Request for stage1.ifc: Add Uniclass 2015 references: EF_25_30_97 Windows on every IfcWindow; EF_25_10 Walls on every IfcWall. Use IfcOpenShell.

First a look at what the model holds.

```python
import ifcopenshell

model = ifcopenshell.open("stage1.ifc")
print(model.schema)
print("classifications:", [c.Name for c in model.by_type("IfcClassification")])
for ifc_class in ("IfcDoor", "IfcRoof", "IfcStair", "IfcWall", "IfcWindow"):
    print(ifc_class, len(model.by_type(ifc_class)))
```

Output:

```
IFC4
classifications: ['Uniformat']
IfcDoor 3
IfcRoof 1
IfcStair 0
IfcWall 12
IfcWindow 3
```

```python
import ifcopenshell
import ifcopenshell.api.classification

model = ifcopenshell.open("stage1.ifc")

system = ifcopenshell.api.classification.add_classification(model, classification="Uniclass 2015")

codes = {
    "IfcWindow": ("EF_25_30_97", "Windows"),
    "IfcWall": ("EF_25_10", "Walls"),
}
for ifc_class, (code, name) in codes.items():
    products = model.by_type(ifc_class)
    ifcopenshell.api.classification.add_reference(
        model, products=products, classification=system, identification=code, name=name
    )
    print(code, len(products))

model.write("stage1_edited.ifc")
```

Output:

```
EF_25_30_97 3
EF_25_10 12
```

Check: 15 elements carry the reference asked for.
